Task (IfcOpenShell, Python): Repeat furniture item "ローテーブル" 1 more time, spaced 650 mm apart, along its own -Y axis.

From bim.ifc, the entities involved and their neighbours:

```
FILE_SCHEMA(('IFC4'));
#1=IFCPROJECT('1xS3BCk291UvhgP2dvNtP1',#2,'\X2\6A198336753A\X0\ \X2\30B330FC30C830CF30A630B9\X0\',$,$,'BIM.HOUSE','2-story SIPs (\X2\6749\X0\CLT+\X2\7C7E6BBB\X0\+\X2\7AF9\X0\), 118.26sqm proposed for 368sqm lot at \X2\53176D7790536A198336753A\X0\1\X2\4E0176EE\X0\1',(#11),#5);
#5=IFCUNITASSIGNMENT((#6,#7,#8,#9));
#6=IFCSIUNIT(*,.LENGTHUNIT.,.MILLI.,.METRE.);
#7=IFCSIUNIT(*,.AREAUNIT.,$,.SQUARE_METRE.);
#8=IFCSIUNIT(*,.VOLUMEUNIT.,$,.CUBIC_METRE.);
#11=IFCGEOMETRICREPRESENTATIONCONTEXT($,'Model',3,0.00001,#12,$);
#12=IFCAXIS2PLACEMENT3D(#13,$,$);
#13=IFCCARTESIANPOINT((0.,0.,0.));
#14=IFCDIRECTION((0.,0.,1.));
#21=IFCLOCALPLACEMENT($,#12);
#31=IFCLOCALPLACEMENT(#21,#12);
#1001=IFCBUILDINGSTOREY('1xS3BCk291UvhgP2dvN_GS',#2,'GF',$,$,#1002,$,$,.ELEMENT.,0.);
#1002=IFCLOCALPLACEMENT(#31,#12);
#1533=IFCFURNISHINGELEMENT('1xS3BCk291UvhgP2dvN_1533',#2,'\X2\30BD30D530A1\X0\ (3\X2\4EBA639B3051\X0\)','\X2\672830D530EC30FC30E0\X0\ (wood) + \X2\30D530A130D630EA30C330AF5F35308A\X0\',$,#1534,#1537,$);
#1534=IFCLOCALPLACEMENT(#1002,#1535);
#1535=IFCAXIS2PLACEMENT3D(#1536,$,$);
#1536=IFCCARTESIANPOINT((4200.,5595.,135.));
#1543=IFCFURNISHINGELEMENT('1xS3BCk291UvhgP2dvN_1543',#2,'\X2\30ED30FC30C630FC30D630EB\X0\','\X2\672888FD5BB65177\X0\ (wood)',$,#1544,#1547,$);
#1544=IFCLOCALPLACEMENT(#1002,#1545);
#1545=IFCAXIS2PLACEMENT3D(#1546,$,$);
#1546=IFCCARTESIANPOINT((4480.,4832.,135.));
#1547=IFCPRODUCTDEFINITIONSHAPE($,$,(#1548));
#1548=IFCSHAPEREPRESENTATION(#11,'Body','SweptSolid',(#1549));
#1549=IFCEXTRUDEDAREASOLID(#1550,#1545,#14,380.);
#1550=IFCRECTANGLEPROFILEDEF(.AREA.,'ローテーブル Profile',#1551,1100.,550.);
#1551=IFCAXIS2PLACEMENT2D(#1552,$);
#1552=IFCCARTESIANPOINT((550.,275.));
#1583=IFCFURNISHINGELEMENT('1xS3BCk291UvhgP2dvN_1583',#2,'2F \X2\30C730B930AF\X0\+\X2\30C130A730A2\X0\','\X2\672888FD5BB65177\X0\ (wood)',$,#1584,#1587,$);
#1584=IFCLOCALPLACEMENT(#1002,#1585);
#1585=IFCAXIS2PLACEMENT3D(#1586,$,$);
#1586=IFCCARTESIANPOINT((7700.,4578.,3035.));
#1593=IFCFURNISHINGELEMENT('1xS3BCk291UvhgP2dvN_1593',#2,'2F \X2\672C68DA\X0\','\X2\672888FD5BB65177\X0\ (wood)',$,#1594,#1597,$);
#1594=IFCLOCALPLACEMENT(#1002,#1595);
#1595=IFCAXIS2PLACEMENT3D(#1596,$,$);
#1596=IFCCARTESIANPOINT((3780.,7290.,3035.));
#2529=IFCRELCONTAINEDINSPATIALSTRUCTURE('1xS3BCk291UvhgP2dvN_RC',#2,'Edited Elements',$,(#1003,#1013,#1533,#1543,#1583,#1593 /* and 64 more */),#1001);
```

```python
import ifcopenshell
import ifcopenshell.api.geometry
import ifcopenshell.api.root
import ifcopenshell.util.element
import ifcopenshell.util.placement
import ifcopenshell.util.unit

model = ifcopenshell.open("bim.ifc")
unit_scale = ifcopenshell.util.unit.calculate_unit_scale(model)


def reuse_history(source, copy):
    """copy_class also copies each property set's owner history, people and application; keep the originals."""
    for rel in copy.IsDefinedBy:
        if rel.is_a("IfcRelDefinesByProperties") and (history := rel.RelatingPropertyDefinition.OwnerHistory):
            rel.RelatingPropertyDefinition.OwnerHistory = source.OwnerHistory
            ifcopenshell.util.element.remove_deep2(model, history)


source = model.by_guid("1xS3BCk291UvhgP2dvN_1543")
base = ifcopenshell.util.placement.get_local_placement(source.ObjectPlacement)
step = -base[:3, 1] * 0.65 / unit_scale

for i in range(1, 2):
    copy = ifcopenshell.api.root.copy_class(model, product=source)
    copy.Representation = ifcopenshell.util.element.copy_deep(
        model, source.Representation, exclude=["IfcGeometricRepresentationContext", "IfcRepresentationMap"]
    )
    reuse_history(source, copy)
    matrix = base.copy()
    matrix[:3, 3] += i * step
    print("added at", matrix[:3, 3].round(3) + 0.0)
    ifcopenshell.api.geometry.edit_object_placement(model, product=copy, matrix=matrix, is_si=False)

model.write("bim_updated.ifc")
```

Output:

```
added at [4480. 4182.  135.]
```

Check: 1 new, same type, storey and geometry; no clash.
